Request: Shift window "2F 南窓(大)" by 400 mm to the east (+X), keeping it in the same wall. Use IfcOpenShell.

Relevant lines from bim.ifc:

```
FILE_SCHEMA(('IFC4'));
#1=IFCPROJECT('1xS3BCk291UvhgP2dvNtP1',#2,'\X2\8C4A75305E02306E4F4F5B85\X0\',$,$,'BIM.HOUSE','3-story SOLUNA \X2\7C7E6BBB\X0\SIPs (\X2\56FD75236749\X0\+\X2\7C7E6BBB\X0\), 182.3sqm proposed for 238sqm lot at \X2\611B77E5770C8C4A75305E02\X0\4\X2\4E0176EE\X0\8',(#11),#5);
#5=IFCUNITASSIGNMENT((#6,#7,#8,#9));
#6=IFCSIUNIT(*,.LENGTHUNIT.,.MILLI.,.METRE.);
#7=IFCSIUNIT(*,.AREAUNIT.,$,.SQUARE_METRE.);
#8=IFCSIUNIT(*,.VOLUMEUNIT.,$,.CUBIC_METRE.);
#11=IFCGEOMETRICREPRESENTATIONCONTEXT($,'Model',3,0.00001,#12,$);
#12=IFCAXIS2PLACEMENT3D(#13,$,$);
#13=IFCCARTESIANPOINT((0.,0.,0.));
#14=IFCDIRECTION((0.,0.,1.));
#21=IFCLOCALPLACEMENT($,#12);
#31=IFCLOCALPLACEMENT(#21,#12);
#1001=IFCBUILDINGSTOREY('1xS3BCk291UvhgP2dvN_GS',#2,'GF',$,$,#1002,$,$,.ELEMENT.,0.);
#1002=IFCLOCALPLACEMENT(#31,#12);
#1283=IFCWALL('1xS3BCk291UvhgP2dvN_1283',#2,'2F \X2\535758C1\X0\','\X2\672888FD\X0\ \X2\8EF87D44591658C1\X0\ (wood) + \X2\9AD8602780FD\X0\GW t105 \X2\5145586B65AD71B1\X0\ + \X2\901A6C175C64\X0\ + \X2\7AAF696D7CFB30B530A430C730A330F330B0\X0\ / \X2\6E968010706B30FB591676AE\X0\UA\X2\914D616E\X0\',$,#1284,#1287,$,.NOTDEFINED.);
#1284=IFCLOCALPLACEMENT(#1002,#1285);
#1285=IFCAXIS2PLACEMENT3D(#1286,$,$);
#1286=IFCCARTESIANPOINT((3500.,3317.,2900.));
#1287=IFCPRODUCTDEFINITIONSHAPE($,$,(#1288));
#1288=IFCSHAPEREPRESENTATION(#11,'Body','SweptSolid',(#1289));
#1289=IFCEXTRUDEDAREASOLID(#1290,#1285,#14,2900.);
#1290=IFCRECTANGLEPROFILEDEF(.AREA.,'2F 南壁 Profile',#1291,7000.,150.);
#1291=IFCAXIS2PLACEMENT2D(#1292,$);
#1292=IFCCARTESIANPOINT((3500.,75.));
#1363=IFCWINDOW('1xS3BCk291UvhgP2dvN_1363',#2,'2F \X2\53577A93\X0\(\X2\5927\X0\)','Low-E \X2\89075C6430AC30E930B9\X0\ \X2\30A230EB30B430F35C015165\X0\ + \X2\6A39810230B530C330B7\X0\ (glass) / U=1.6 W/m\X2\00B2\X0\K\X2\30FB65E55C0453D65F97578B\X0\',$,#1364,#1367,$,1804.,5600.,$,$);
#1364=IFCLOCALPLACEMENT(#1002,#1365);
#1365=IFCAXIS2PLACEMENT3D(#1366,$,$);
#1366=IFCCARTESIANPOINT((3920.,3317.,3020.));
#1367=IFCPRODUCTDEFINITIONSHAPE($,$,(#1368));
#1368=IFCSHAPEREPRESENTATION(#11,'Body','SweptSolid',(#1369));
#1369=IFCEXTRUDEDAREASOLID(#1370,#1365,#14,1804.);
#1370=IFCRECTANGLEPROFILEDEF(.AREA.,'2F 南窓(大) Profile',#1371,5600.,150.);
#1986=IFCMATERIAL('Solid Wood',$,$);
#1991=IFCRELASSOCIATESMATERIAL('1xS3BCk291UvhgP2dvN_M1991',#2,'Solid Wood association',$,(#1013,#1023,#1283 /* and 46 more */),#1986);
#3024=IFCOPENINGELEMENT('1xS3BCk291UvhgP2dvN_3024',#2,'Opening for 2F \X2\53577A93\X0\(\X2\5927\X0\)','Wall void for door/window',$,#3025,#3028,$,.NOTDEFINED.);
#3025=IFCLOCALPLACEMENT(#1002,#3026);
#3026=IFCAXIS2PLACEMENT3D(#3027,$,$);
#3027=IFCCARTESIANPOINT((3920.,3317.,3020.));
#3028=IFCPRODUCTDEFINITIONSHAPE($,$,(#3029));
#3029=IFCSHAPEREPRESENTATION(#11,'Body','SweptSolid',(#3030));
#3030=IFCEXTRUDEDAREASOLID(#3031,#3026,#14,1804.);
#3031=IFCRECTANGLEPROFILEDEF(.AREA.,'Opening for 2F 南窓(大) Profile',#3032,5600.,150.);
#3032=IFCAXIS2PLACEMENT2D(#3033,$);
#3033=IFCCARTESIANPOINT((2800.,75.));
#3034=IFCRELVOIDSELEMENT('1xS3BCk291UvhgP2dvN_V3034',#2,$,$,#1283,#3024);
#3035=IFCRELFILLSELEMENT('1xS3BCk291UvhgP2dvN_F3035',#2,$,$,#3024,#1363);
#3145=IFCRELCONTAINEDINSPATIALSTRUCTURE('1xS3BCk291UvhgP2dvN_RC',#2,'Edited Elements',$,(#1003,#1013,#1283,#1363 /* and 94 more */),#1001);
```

```python
import ifcopenshell
import ifcopenshell.api.geometry
import ifcopenshell.util.placement
import ifcopenshell.util.unit

model = ifcopenshell.open("bim.ifc")
unit_scale = ifcopenshell.util.unit.calculate_unit_scale(model)

window = model.by_id(1363)
opening = window.FillsVoids[0].RelatingOpeningElement
wall = opening.VoidsElements[0].RelatingBuildingElement

wall_matrix = ifcopenshell.util.placement.get_local_placement(wall.ObjectPlacement)
shift = wall_matrix[:3, 0] * 0.4 / unit_scale
before = ifcopenshell.util.placement.get_local_placement(window.ObjectPlacement)[:3, 3].copy()

# The window is not placed relative to its opening, so move both.
for product in (opening, window):
    matrix = ifcopenshell.util.placement.get_local_placement(product.ObjectPlacement)
    matrix[:3, 3] += shift
    ifcopenshell.api.geometry.edit_object_placement(model, product=product, matrix=matrix, is_si=False)

after = ifcopenshell.util.placement.get_local_placement(window.ObjectPlacement)[:3, 3]
print("window moved by", (after - before).round(3) + 0.0)

model.write("bim-out.ifc")
```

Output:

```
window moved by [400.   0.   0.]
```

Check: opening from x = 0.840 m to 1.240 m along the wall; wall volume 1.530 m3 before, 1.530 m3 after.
